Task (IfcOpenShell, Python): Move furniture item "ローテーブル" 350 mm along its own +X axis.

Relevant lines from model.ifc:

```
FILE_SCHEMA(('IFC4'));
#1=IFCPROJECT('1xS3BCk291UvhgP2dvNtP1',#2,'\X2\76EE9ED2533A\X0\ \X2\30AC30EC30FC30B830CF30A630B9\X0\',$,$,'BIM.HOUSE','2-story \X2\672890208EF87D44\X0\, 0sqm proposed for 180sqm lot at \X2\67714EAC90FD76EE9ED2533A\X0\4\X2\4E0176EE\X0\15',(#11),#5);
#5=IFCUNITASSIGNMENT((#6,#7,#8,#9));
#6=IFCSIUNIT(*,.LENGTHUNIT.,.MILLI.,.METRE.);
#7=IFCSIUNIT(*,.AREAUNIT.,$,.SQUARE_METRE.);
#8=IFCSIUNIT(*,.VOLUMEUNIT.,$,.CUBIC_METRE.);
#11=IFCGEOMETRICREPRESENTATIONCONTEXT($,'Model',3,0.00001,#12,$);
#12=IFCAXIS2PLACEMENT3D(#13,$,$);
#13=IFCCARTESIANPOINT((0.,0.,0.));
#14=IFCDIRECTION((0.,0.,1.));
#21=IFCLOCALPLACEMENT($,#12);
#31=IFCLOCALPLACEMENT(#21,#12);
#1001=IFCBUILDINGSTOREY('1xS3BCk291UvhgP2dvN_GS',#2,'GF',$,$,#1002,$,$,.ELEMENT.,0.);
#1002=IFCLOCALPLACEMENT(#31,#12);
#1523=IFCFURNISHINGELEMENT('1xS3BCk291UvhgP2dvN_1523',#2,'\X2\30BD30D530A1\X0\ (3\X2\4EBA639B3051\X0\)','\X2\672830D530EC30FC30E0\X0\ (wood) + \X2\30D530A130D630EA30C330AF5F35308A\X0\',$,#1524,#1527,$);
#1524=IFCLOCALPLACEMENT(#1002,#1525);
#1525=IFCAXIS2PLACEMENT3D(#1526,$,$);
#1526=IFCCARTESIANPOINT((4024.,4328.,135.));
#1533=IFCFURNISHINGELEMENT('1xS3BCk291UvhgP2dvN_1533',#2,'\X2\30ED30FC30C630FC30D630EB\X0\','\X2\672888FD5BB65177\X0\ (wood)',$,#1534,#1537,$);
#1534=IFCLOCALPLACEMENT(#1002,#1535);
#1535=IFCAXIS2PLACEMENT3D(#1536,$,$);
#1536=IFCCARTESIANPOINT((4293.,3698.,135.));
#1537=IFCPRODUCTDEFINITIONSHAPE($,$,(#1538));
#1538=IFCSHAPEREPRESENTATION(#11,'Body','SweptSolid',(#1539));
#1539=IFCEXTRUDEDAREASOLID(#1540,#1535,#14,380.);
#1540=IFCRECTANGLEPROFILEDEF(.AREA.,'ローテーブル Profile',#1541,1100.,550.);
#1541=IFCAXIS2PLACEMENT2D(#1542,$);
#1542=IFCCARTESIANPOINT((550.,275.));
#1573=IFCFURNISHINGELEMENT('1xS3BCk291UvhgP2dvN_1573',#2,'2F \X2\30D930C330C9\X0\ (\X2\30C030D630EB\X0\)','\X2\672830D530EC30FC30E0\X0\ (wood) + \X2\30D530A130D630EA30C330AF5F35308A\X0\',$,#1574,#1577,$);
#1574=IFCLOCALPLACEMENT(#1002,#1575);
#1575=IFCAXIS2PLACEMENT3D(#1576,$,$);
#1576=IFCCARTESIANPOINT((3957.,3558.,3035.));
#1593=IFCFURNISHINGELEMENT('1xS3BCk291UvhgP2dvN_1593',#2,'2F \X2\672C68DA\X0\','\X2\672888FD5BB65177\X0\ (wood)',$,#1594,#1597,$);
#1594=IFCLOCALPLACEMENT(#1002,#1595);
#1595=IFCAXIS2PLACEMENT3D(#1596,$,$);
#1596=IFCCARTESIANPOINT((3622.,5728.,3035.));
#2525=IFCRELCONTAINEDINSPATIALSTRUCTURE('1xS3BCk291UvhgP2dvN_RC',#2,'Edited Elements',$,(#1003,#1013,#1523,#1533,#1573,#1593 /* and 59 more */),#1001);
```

```python
import ifcopenshell
import ifcopenshell.api.geometry
import ifcopenshell.util.placement

model = ifcopenshell.open("model.ifc")

item = model.by_guid("1xS3BCk291UvhgP2dvN_1533")
matrix = ifcopenshell.util.placement.get_local_placement(item.ObjectPlacement)
matrix[:3, 3] += matrix[:3, 0] * 350.0
ifcopenshell.api.geometry.edit_object_placement(model, product=item, matrix=matrix, is_si=False)

print(ifcopenshell.util.placement.get_local_placement(item.ObjectPlacement).round(3) + 0.0)

model.write("model_v2.ifc")
```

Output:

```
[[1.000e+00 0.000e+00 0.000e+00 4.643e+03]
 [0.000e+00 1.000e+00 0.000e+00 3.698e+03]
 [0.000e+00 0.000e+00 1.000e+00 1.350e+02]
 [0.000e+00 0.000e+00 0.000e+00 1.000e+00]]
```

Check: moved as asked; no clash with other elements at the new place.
